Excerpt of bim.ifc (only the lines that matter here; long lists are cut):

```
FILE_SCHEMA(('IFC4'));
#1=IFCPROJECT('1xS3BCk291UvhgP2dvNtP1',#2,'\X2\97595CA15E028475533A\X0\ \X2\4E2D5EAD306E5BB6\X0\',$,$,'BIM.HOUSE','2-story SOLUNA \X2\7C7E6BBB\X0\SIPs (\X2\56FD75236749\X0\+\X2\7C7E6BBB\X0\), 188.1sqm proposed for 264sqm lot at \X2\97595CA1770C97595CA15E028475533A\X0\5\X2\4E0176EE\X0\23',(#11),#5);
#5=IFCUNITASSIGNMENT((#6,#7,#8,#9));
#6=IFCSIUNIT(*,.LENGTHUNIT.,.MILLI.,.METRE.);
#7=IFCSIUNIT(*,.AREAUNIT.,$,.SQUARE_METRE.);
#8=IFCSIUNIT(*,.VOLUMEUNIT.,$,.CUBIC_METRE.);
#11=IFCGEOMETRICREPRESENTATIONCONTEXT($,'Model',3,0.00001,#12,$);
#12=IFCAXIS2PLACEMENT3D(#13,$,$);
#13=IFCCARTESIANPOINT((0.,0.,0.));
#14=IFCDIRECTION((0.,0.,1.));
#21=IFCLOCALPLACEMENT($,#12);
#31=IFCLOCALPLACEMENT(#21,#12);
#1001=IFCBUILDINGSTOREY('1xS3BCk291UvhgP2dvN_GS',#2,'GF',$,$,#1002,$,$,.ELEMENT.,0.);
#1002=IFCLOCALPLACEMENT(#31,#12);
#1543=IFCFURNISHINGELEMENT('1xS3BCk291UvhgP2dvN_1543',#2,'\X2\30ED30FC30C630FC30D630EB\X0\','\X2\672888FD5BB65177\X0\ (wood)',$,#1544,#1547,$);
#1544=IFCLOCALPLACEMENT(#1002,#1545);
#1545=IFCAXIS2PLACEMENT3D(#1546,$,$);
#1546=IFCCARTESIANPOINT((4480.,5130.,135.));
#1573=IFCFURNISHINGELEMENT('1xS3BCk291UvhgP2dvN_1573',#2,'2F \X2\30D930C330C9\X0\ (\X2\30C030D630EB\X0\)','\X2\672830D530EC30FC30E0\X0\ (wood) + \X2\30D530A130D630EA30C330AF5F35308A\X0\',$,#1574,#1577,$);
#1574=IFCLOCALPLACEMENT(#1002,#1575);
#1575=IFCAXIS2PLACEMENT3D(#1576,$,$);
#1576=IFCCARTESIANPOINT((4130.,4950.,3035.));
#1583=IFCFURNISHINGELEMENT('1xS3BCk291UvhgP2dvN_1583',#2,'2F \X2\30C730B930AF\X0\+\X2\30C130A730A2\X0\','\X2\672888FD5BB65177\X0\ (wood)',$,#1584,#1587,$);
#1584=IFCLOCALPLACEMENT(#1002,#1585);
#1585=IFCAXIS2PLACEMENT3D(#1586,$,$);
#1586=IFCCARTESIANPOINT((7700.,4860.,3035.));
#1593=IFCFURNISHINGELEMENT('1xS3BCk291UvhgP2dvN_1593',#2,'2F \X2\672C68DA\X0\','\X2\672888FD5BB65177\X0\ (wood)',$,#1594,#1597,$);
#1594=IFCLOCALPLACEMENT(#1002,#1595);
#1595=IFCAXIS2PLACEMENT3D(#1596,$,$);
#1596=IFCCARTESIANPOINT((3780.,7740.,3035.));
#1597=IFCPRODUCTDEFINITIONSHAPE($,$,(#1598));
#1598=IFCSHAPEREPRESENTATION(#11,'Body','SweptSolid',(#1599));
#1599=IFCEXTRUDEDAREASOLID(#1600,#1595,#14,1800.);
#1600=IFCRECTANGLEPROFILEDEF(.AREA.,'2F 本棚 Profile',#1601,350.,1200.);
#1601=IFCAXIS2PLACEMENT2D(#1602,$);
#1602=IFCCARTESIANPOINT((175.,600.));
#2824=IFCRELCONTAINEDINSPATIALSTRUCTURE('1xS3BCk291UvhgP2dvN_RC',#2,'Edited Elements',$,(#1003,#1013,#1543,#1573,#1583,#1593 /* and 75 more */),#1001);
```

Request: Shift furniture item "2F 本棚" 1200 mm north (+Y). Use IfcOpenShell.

```python
import ifcopenshell
import ifcopenshell.api.geometry
import ifcopenshell.util.placement
import ifcopenshell.util.unit

model = ifcopenshell.open("bim.ifc")
unit_scale = ifcopenshell.util.unit.calculate_unit_scale(model)

item = model.by_guid("1xS3BCk291UvhgP2dvN_1593")
matrix = ifcopenshell.util.placement.get_local_placement(item.ObjectPlacement)
matrix[1, 3] += 1.2 / unit_scale
ifcopenshell.api.geometry.edit_object_placement(model, product=item, matrix=matrix, is_si=False)

print(ifcopenshell.util.placement.get_local_placement(item.ObjectPlacement).round(3) + 0.0)

model.write("bim_rev.ifc")
```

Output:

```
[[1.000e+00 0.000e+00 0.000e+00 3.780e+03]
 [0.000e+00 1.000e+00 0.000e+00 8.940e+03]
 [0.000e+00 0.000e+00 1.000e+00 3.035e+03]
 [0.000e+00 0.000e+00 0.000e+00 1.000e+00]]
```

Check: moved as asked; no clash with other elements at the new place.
